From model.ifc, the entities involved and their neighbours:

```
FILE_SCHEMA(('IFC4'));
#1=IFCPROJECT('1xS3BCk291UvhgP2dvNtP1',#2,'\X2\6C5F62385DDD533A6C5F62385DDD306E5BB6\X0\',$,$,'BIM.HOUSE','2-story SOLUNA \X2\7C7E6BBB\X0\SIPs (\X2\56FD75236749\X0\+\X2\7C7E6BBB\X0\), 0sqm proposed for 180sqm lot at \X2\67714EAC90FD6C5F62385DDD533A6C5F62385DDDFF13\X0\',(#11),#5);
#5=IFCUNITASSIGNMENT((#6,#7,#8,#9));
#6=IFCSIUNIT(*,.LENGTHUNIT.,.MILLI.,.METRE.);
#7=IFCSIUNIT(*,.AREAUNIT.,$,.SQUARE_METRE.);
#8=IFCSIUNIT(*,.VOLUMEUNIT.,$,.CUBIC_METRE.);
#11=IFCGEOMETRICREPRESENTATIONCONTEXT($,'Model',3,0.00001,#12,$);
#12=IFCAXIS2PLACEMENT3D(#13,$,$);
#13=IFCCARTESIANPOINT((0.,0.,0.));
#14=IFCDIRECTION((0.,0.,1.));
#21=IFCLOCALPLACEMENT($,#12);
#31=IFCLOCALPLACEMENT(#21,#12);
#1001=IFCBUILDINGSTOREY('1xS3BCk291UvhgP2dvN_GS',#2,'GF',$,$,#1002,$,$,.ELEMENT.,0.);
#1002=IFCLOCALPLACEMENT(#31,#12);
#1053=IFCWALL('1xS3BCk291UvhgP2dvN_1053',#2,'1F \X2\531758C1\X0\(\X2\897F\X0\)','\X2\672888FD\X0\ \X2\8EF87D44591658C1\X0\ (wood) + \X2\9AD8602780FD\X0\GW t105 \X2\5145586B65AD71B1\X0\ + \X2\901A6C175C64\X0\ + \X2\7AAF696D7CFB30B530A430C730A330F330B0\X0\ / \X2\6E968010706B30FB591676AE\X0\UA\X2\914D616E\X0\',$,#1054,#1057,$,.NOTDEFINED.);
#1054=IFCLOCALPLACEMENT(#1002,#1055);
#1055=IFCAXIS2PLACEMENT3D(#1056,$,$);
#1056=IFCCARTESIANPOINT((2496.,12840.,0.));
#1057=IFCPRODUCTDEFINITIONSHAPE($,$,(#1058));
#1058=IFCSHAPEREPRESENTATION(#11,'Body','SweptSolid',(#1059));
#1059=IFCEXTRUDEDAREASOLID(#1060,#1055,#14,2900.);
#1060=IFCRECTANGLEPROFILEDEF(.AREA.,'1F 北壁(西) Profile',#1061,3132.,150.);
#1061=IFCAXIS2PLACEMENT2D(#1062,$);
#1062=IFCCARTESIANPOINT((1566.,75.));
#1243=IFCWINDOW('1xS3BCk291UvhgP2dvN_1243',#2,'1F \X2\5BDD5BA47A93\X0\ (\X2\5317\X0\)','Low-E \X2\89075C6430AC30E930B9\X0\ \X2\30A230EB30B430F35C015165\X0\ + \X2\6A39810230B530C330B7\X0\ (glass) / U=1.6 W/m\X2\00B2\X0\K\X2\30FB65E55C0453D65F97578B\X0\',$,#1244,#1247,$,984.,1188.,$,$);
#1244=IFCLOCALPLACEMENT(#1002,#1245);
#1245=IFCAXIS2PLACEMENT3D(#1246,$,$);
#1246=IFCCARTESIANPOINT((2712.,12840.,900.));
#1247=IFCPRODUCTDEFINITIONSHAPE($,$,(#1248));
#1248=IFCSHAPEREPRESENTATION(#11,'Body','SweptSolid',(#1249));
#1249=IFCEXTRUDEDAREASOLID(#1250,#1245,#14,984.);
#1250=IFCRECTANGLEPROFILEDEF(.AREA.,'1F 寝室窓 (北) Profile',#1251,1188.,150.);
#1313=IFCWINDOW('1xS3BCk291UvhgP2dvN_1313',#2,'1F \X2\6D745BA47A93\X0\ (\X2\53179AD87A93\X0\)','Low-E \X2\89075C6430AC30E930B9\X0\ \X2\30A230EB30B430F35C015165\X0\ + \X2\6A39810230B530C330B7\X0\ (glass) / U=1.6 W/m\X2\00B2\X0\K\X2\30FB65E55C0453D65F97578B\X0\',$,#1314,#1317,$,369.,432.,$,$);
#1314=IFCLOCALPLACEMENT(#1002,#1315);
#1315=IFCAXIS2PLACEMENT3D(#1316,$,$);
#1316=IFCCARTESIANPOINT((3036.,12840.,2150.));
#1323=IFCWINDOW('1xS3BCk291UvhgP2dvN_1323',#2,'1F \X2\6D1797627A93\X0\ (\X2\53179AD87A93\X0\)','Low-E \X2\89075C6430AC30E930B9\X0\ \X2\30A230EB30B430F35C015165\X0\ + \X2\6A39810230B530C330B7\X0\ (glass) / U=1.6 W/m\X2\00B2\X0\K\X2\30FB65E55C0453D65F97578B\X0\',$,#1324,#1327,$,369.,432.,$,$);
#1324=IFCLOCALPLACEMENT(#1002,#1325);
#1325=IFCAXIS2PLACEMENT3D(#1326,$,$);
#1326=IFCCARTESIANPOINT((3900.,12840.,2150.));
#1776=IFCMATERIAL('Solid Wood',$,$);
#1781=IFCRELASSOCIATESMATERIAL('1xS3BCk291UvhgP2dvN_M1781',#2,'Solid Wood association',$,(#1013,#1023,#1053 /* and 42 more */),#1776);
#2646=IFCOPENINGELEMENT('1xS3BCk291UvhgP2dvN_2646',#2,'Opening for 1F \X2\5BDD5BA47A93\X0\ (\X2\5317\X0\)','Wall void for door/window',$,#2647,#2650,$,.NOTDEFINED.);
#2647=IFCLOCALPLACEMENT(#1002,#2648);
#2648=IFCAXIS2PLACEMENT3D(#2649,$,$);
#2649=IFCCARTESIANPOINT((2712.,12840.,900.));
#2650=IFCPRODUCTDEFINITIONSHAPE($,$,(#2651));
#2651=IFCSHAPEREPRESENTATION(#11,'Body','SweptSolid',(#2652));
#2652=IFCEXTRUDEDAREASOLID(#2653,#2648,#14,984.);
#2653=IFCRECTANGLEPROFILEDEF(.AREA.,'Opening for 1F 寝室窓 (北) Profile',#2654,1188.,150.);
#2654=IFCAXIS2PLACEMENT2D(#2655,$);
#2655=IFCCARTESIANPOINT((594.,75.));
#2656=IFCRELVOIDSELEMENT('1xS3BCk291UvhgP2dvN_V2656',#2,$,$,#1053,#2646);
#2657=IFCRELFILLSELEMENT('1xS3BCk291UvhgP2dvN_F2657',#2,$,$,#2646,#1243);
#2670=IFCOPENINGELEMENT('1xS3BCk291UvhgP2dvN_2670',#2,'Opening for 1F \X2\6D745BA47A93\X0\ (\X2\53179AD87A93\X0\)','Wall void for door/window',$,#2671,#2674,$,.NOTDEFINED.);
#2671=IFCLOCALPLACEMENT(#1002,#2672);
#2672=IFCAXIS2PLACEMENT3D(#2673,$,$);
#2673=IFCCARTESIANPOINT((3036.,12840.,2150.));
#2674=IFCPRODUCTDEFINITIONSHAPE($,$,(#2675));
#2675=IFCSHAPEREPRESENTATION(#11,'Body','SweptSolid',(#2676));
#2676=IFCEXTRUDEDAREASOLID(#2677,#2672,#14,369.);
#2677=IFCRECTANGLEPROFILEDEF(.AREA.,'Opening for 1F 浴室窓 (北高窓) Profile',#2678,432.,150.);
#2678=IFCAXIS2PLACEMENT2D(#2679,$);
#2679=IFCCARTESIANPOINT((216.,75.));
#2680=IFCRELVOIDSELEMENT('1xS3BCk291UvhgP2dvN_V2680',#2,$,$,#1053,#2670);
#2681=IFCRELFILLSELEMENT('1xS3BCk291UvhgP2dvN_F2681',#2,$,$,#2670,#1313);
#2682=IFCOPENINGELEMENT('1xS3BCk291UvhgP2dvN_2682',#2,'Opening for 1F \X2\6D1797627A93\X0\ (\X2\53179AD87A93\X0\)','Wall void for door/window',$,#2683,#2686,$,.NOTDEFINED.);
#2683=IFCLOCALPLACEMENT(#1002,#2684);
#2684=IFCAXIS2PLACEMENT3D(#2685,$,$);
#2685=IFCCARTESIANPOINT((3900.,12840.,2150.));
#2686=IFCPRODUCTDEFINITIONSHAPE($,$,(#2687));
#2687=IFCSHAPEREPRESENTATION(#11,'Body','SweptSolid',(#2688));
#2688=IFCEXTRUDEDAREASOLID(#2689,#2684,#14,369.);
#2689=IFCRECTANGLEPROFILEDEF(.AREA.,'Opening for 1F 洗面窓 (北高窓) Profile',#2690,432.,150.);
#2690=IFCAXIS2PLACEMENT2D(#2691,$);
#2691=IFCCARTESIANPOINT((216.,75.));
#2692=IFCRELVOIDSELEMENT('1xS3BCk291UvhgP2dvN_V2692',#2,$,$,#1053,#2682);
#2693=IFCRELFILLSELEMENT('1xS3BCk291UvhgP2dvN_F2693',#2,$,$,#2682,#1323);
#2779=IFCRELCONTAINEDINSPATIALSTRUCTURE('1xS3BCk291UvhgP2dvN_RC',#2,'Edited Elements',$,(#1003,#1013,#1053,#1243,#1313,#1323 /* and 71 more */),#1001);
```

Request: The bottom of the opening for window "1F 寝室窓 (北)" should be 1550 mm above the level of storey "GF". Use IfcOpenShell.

```python
import numpy as np
import ifcopenshell
import ifcopenshell.api.geometry
import ifcopenshell.geom
import ifcopenshell.util.element
import ifcopenshell.util.placement
import ifcopenshell.util.shape
import ifcopenshell.util.unit

model = ifcopenshell.open("model.ifc")
unit_scale = ifcopenshell.util.unit.calculate_unit_scale(model)

window = model.by_guid("1xS3BCk291UvhgP2dvN_1243")
opening = window.FillsVoids[0].RelatingOpeningElement
storey = ifcopenshell.util.element.get_container(window, ifc_class="IfcBuildingStorey")
level = ifcopenshell.util.placement.get_local_placement(storey.ObjectPlacement)[2, 3]

# The opening's origin need not be at the sill, so measure its lowest point.
shape = ifcopenshell.geom.create_shape(ifcopenshell.geom.settings(), opening)
bottom = ifcopenshell.util.shape.get_shape_bottom_elevation(shape, shape.geometry) / unit_scale
dz = level + 1.55 / unit_scale - bottom

shift = np.array([0.0, 0.0, dz])
# The window is not placed relative to its opening, so move both.
for product in (opening, window):
    matrix = ifcopenshell.util.placement.get_local_placement(product.ObjectPlacement)
    matrix[:3, 3] += shift
    ifcopenshell.api.geometry.edit_object_placement(model, product=product, matrix=matrix, is_si=False)

print(f"moved by {dz * unit_scale:+.3f} m")

model.write("model_updated.ifc")
```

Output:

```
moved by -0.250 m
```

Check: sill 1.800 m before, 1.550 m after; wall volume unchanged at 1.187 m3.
